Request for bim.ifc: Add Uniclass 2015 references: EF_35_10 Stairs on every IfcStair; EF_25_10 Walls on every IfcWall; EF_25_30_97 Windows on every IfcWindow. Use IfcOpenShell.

First a look at what the model holds.

```python
import ifcopenshell

model = ifcopenshell.open("bim.ifc")
print(model.schema)
print("classifications:", [c.Name for c in model.by_type("IfcClassification")])
for ifc_class in ("IfcDoor", "IfcRoof", "IfcStair", "IfcWall", "IfcWindow"):
    print(ifc_class, len(model.by_type(ifc_class)))
```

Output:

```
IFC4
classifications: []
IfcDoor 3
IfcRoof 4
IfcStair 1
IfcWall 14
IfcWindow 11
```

```python
import ifcopenshell
import ifcopenshell.api.classification

model = ifcopenshell.open("bim.ifc")

system = ifcopenshell.api.classification.add_classification(model, classification="Uniclass 2015")

codes = {
    "IfcStair": ("EF_35_10", "Stairs"),
    "IfcWall": ("EF_25_10", "Walls"),
    "IfcWindow": ("EF_25_30_97", "Windows"),
}
for ifc_class, (code, name) in codes.items():
    products = model.by_type(ifc_class)
    ifcopenshell.api.classification.add_reference(
        model, products=products, classification=system, identification=code, name=name
    )
    print(code, len(products))

model.write("bim_v2.ifc")
```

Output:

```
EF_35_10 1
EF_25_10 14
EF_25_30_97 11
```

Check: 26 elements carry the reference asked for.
